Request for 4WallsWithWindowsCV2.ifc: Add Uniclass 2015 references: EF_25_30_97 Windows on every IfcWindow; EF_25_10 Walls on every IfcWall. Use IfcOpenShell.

First a look at what the model holds.

```python
import ifcopenshell

model = ifcopenshell.open("4WallsWithWindowsCV2.ifc")
print(model.schema)
print("classifications:", [c.Name for c in model.by_type("IfcClassification")])
for ifc_class in ("IfcDoor", "IfcRoof", "IfcStair", "IfcWall", "IfcWindow"):
    print(ifc_class, len(model.by_type(ifc_class)))
```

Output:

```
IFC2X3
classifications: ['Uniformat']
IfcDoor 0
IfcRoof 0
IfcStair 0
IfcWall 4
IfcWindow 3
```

```python
import ifcopenshell
import ifcopenshell.api.classification

model = ifcopenshell.open("4WallsWithWindowsCV2.ifc")

# IFC2X3 requires Source and Edition and has no link from the project to the system.
system = model.create_entity("IfcClassification", Source="NBS", Edition="2015", Name="Uniclass 2015")

codes = {
    "IfcWindow": ("EF_25_30_97", "Windows"),
    "IfcWall": ("EF_25_10", "Walls"),
}
for ifc_class, (code, name) in codes.items():
    products = model.by_type(ifc_class)
    ifcopenshell.api.classification.add_reference(
        model, products=products, classification=system, identification=code, name=name
    )
    print(code, len(products))

model.write("4WallsWithWindowsCV2_v2.ifc")
```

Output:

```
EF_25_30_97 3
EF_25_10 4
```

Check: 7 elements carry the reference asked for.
